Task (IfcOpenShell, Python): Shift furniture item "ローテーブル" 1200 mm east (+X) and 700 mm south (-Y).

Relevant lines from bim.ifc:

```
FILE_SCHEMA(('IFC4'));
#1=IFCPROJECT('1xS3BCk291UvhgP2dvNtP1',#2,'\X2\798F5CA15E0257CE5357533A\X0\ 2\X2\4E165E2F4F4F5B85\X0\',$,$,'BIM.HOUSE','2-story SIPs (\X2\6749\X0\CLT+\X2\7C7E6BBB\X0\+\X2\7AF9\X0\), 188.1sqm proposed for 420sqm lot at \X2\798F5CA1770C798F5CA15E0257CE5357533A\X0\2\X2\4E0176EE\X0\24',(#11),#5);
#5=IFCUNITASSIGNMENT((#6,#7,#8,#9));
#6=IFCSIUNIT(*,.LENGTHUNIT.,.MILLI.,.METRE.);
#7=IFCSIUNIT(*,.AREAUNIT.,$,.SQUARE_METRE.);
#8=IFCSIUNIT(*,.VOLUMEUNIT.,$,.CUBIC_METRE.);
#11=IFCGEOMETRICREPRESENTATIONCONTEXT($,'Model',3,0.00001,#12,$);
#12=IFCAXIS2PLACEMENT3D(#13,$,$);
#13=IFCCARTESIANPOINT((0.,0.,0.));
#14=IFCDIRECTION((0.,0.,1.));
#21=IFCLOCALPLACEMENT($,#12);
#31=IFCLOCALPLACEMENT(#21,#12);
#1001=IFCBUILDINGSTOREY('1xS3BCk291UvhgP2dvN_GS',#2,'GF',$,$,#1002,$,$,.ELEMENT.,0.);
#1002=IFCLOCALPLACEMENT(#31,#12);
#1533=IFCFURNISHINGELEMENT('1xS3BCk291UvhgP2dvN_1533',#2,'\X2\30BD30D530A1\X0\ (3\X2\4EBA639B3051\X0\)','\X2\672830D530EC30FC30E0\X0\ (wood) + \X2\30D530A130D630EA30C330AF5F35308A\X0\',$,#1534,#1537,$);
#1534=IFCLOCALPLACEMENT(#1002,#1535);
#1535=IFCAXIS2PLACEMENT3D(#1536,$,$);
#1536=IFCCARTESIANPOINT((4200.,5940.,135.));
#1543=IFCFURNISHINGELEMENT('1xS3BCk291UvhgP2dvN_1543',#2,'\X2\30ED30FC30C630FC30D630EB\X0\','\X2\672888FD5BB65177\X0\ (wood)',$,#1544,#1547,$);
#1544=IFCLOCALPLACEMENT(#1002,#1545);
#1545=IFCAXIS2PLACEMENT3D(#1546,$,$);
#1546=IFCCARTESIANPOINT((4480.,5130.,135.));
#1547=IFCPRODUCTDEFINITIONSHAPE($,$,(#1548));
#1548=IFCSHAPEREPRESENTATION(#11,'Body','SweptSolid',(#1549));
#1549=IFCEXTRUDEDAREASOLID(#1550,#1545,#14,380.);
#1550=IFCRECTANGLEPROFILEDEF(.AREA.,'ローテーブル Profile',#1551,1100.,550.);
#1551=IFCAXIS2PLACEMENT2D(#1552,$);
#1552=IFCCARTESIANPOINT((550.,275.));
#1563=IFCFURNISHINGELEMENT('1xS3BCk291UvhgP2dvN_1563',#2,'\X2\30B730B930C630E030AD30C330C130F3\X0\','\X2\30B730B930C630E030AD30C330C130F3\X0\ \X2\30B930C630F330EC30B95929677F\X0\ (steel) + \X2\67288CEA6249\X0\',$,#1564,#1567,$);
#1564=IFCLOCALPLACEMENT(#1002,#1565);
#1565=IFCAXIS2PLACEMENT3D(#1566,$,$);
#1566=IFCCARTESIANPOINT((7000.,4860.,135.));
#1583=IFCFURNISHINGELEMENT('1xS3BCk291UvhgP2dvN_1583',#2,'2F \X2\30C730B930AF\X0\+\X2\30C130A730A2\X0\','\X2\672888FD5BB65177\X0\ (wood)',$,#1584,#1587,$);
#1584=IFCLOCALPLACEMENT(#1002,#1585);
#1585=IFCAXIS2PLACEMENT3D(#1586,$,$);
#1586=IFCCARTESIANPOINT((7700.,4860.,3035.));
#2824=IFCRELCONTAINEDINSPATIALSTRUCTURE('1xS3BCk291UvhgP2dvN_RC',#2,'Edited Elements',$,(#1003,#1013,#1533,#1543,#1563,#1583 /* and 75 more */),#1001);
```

```python
import ifcopenshell
import ifcopenshell.api.geometry
import ifcopenshell.util.placement

model = ifcopenshell.open("bim.ifc")

item = model.by_id(1543)
matrix = ifcopenshell.util.placement.get_local_placement(item.ObjectPlacement)
matrix[0, 3] += 1200.0
matrix[1, 3] -= 700.0
ifcopenshell.api.geometry.edit_object_placement(model, product=item, matrix=matrix, is_si=False)

print(ifcopenshell.util.placement.get_local_placement(item.ObjectPlacement).round(3) + 0.0)

model.write("bim_updated.ifc")
```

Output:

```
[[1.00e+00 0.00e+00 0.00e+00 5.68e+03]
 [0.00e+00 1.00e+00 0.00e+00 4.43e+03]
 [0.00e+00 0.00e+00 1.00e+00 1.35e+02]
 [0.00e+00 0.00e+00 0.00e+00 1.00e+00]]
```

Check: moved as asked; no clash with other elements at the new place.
